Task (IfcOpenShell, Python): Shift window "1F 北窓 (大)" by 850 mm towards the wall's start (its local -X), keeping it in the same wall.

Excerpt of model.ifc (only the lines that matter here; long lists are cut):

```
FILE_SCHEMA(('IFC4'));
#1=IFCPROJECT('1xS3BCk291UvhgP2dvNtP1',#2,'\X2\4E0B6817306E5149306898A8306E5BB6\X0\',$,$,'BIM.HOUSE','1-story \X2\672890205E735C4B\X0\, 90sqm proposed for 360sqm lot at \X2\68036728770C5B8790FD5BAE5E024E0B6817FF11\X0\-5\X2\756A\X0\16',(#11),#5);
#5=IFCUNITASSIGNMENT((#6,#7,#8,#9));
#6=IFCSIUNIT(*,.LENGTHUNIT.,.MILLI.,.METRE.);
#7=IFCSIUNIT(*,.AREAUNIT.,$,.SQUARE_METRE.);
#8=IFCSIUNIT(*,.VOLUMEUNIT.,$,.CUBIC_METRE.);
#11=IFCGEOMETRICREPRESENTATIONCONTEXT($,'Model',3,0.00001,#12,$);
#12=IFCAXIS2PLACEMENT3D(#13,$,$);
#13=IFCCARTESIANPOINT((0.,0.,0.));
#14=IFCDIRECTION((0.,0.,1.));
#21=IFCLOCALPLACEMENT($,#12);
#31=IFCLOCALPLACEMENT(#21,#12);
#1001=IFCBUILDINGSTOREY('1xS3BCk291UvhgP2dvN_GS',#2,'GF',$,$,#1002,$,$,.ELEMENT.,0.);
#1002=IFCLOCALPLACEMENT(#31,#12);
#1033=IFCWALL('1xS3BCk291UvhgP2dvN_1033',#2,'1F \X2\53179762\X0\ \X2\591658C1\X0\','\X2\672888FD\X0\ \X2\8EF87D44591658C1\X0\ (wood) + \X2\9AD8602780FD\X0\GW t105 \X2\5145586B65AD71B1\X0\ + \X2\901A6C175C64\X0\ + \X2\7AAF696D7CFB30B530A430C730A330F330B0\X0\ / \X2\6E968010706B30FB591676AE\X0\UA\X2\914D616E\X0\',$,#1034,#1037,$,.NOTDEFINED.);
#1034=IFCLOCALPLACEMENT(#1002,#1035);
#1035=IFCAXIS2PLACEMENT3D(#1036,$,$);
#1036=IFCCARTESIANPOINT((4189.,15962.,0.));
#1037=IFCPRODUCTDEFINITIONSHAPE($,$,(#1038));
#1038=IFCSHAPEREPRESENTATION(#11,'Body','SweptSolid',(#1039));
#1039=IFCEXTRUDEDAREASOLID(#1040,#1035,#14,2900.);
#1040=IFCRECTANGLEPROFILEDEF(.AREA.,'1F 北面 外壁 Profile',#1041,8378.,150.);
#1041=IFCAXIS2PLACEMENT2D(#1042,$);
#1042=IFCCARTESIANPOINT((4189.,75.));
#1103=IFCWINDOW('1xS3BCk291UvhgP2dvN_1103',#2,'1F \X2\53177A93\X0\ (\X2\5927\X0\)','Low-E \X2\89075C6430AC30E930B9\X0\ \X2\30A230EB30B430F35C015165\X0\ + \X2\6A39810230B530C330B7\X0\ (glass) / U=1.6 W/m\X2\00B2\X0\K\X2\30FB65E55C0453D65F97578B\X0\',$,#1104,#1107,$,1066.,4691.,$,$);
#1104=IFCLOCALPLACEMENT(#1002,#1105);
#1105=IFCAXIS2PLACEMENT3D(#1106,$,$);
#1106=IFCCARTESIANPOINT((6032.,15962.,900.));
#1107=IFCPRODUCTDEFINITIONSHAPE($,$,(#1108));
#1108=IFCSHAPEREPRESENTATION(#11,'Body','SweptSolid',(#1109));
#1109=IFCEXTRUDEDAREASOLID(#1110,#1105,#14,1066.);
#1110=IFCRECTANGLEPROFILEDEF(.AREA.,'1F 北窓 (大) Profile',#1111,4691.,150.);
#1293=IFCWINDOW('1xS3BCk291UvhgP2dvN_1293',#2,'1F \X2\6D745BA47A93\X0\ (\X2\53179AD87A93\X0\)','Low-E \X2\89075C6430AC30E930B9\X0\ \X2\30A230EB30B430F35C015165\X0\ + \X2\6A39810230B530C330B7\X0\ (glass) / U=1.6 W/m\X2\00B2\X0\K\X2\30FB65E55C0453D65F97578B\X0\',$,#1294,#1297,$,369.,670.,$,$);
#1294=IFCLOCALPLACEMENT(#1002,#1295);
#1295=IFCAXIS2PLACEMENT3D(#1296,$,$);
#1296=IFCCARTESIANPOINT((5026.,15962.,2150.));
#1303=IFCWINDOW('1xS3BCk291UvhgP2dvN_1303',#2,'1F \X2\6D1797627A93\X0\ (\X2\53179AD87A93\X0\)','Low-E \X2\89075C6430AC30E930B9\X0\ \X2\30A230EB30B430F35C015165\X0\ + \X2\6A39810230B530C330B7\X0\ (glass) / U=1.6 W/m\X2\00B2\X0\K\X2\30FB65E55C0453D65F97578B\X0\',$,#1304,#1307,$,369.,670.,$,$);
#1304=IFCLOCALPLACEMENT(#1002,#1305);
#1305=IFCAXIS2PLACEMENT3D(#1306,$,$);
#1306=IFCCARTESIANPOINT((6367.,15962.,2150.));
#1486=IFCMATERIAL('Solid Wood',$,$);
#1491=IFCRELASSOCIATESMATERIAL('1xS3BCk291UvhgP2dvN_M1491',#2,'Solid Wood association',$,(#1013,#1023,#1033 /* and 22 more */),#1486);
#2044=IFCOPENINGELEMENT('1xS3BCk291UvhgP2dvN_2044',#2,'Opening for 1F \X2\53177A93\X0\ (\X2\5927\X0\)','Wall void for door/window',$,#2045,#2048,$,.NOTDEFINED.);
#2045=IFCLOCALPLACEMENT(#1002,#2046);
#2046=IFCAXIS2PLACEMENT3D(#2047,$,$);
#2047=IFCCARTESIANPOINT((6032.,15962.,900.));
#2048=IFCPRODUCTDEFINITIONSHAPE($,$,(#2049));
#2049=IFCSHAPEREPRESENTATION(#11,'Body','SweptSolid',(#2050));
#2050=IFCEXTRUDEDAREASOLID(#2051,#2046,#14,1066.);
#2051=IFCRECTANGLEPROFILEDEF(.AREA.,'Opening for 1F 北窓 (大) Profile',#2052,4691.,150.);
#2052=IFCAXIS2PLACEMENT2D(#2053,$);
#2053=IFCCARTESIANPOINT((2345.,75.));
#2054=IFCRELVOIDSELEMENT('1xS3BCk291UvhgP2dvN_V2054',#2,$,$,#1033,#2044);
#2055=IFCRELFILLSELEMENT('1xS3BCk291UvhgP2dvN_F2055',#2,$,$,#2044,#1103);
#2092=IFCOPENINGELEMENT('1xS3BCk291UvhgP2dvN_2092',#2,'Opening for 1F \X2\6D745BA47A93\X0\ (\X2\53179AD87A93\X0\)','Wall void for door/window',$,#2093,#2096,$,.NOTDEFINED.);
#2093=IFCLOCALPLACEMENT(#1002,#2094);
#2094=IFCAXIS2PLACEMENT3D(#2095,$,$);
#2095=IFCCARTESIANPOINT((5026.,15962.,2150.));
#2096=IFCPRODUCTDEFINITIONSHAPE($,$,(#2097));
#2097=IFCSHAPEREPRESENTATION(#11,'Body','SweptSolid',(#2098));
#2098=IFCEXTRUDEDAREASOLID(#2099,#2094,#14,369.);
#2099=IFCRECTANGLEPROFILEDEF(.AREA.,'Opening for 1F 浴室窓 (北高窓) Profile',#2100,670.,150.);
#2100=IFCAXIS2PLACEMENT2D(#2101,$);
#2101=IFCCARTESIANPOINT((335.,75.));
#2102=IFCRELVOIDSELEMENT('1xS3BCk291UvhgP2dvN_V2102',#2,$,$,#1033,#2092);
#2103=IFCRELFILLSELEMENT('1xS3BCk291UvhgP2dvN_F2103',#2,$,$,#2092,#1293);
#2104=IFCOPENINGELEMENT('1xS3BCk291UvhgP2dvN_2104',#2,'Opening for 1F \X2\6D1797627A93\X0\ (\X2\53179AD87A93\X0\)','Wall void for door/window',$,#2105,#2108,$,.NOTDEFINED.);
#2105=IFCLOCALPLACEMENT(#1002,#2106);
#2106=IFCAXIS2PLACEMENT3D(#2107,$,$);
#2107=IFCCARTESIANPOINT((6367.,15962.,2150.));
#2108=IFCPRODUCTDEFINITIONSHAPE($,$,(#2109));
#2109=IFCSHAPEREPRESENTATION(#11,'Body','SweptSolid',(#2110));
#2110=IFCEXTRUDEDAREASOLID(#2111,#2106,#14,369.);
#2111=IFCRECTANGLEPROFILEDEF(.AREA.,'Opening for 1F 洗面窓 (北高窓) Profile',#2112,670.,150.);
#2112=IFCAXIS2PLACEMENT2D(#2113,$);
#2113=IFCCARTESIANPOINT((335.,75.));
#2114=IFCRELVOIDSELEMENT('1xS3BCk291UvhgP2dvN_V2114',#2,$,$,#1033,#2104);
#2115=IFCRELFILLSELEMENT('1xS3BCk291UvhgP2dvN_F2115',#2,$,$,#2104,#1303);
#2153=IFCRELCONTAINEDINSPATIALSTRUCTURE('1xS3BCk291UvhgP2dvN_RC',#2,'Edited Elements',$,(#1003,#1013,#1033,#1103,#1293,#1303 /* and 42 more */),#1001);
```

```python
import ifcopenshell
import ifcopenshell.api.geometry
import ifcopenshell.util.placement

model = ifcopenshell.open("model.ifc")

window = model.by_id(1103)
opening = window.FillsVoids[0].RelatingOpeningElement
wall = opening.VoidsElements[0].RelatingBuildingElement

wall_matrix = ifcopenshell.util.placement.get_local_placement(wall.ObjectPlacement)
shift = wall_matrix[:3, 0] * -850.0
before = ifcopenshell.util.placement.get_local_placement(window.ObjectPlacement)[:3, 3].copy()

# The window is not placed relative to its opening, so move both.
for product in (opening, window):
    matrix = ifcopenshell.util.placement.get_local_placement(product.ObjectPlacement)
    matrix[:3, 3] += shift
    ifcopenshell.api.geometry.edit_object_placement(model, product=product, matrix=matrix, is_si=False)

after = ifcopenshell.util.placement.get_local_placement(window.ObjectPlacement)[:3, 3]
print("window moved by", (after - before).round(3) + 0.0)

model.write("model-out.ifc")
```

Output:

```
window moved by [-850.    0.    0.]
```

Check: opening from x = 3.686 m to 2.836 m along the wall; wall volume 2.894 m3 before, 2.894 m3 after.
